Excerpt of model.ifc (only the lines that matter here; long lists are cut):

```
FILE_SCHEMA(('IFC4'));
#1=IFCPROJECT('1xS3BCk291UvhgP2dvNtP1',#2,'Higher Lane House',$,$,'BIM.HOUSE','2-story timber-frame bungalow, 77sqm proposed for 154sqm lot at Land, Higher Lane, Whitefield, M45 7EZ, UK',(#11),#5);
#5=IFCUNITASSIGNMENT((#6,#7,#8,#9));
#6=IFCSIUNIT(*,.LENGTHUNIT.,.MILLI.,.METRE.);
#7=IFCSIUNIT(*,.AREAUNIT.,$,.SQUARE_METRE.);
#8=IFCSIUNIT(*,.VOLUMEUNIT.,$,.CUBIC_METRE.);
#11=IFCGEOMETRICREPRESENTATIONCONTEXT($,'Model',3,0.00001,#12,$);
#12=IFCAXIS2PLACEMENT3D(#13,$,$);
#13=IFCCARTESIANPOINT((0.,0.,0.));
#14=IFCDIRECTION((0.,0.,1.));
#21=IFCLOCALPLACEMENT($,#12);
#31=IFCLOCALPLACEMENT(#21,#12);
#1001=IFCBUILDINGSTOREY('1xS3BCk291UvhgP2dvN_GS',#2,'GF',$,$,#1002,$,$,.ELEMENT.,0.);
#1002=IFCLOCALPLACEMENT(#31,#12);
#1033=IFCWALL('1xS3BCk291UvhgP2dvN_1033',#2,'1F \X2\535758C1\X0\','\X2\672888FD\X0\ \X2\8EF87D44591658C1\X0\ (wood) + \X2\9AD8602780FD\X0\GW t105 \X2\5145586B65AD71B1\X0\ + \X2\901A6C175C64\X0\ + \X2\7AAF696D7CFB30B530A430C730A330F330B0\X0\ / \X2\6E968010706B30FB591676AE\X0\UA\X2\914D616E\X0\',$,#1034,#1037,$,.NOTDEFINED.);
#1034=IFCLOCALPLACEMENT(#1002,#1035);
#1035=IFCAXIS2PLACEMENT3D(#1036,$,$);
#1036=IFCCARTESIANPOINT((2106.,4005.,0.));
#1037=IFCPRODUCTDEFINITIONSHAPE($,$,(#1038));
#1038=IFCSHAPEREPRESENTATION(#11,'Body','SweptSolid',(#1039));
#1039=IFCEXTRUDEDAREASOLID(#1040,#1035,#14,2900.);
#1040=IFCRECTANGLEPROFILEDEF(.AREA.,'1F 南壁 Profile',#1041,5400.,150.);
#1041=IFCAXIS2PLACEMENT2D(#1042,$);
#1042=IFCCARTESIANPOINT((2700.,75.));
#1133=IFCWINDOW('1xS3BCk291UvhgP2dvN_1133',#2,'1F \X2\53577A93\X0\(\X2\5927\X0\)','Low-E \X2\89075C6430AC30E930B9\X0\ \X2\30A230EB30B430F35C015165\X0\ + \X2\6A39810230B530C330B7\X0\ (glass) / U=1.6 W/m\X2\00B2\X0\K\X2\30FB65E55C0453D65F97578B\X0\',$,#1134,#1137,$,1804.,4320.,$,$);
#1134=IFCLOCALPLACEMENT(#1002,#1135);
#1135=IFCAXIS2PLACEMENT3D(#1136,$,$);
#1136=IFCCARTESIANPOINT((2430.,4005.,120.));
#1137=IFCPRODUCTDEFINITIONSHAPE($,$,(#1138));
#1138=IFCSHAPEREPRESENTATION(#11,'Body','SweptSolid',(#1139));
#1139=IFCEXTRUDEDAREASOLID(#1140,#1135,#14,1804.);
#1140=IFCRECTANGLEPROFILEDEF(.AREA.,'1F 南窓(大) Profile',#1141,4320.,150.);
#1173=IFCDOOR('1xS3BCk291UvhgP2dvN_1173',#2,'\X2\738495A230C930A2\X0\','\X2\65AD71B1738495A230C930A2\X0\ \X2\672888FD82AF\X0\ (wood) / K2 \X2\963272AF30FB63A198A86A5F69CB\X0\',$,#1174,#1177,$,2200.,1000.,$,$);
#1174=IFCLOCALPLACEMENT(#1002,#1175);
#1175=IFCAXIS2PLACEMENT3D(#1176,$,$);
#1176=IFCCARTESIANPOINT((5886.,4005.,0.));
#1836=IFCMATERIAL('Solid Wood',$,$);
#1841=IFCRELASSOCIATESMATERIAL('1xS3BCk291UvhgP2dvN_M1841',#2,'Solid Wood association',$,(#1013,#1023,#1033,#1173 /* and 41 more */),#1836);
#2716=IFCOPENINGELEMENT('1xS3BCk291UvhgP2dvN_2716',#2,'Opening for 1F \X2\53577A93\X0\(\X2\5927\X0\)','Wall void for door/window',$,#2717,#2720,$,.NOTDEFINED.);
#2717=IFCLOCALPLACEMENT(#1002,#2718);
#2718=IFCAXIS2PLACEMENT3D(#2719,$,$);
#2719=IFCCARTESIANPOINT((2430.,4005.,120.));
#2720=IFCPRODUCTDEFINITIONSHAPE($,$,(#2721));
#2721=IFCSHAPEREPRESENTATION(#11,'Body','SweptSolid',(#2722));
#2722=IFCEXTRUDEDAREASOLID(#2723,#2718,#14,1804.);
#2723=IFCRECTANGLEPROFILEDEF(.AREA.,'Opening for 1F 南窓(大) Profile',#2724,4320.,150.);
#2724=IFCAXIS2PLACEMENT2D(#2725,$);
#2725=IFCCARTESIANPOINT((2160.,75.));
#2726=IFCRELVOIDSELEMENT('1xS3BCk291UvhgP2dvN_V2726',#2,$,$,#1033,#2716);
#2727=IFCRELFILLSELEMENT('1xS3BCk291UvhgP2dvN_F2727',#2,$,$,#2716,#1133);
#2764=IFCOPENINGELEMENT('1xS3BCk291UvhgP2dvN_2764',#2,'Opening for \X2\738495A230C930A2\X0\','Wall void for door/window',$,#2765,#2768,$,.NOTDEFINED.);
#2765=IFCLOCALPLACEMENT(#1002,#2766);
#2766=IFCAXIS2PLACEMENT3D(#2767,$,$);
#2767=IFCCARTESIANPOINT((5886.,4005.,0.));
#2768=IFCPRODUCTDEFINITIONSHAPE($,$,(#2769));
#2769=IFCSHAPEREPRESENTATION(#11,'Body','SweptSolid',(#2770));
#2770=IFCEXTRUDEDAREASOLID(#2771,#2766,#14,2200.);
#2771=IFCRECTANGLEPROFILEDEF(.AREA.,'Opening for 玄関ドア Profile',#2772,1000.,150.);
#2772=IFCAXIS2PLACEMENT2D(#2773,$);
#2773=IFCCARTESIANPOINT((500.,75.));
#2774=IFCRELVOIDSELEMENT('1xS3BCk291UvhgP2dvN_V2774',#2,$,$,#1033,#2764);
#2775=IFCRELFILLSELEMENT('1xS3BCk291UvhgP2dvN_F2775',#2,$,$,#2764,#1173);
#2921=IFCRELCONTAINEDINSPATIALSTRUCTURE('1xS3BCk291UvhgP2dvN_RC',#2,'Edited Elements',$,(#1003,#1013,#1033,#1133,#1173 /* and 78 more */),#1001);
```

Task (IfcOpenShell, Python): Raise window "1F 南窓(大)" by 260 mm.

```python
import numpy as np
import ifcopenshell
import ifcopenshell.api.geometry
import ifcopenshell.util.placement
import ifcopenshell.util.unit

model = ifcopenshell.open("model.ifc")
unit_scale = ifcopenshell.util.unit.calculate_unit_scale(model)

window = model.by_id(1133)
opening = window.FillsVoids[0].RelatingOpeningElement
dz = 260.0

shift = np.array([0.0, 0.0, dz])
# The window is not placed relative to its opening, so move both.
for product in (opening, window):
    matrix = ifcopenshell.util.placement.get_local_placement(product.ObjectPlacement)
    matrix[:3, 3] += shift
    ifcopenshell.api.geometry.edit_object_placement(model, product=product, matrix=matrix, is_si=False)

print(f"moved by {dz * unit_scale:+.3f} m")

model.write("model_edited.ifc")
```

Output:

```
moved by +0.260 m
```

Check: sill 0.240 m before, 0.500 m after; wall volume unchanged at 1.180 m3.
